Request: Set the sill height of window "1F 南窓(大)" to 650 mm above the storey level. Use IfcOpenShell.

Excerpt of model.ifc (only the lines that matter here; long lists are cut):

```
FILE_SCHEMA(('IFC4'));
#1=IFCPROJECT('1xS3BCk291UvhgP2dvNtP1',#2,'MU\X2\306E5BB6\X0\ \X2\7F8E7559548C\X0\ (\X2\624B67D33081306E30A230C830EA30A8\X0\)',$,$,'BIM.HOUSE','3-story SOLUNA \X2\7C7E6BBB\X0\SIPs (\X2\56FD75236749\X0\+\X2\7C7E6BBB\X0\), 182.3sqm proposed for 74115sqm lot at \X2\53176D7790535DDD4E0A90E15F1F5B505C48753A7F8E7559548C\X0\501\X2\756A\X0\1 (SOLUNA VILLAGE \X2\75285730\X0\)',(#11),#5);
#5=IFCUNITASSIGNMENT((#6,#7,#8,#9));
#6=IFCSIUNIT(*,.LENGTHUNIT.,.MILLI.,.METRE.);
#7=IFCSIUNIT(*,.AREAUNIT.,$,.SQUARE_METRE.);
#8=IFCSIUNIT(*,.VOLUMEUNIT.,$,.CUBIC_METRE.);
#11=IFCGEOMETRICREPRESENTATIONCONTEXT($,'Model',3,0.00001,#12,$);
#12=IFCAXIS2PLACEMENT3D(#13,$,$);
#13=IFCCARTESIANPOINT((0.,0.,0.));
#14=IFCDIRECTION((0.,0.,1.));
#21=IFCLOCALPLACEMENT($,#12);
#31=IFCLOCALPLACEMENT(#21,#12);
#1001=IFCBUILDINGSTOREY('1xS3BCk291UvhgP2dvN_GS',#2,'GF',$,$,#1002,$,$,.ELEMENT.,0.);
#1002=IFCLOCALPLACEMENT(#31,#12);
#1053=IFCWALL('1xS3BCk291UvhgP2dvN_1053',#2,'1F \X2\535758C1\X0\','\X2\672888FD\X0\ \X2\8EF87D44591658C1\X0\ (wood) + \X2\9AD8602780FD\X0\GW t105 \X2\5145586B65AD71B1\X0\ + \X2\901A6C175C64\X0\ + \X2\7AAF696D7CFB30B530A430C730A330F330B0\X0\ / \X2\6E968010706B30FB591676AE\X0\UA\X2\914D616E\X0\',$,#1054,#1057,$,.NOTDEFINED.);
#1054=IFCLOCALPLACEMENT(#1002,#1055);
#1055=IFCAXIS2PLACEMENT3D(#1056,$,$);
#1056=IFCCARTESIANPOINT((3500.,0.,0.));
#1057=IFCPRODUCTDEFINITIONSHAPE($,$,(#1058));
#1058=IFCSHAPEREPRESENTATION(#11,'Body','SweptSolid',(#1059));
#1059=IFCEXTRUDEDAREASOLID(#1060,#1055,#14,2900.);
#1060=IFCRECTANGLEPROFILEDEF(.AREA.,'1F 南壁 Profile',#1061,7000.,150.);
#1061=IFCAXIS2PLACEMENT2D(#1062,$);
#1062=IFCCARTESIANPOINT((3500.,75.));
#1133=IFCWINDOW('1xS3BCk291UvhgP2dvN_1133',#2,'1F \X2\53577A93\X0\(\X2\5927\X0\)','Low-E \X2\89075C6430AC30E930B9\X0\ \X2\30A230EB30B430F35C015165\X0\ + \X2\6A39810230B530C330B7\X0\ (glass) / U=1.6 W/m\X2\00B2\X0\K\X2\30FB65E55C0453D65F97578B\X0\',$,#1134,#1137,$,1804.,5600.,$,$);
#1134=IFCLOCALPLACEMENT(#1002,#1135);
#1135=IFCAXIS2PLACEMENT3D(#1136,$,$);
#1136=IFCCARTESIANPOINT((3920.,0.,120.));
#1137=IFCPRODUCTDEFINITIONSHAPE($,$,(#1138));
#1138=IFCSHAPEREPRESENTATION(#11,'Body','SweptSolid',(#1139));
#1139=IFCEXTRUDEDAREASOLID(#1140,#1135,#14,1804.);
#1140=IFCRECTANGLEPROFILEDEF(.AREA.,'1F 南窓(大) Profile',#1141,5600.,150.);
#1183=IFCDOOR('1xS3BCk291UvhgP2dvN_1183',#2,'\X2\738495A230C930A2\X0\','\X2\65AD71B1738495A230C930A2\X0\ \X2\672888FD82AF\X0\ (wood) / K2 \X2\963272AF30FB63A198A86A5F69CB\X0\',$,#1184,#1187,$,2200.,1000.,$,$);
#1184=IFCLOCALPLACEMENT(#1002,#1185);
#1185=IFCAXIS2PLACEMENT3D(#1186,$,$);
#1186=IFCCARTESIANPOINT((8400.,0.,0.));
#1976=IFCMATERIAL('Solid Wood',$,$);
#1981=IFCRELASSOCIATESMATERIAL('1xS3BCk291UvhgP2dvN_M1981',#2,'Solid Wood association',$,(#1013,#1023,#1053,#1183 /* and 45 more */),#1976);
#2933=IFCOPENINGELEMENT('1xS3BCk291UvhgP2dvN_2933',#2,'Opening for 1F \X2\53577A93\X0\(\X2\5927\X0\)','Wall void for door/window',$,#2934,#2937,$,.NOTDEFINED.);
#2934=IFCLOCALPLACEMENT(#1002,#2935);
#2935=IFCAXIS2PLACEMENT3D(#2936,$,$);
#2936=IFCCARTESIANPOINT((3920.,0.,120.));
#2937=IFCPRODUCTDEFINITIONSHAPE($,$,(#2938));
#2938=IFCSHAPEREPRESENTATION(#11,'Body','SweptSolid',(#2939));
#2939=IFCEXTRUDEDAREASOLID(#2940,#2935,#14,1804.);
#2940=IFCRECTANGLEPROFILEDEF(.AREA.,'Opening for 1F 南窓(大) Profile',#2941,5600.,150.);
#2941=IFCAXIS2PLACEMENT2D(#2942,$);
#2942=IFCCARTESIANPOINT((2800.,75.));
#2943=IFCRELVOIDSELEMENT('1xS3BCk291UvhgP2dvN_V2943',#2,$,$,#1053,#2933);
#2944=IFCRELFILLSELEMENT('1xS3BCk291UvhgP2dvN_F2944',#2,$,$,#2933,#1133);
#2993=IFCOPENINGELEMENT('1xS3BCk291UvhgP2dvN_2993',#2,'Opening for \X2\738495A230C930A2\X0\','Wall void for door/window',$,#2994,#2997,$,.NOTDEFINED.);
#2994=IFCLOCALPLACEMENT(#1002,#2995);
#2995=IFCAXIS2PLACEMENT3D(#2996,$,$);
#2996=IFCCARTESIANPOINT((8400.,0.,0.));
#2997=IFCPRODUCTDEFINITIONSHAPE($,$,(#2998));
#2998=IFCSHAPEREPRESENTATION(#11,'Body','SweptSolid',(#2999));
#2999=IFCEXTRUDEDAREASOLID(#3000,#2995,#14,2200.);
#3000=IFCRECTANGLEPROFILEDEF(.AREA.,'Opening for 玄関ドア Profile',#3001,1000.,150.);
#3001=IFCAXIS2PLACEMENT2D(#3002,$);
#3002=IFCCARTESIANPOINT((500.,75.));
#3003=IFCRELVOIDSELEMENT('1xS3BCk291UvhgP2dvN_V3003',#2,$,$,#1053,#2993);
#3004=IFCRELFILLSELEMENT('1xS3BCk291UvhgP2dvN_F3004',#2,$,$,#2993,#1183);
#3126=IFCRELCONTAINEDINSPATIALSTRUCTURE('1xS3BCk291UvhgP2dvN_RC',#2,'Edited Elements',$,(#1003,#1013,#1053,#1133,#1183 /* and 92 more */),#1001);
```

```python
import numpy as np
import ifcopenshell
import ifcopenshell.api.geometry
import ifcopenshell.geom
import ifcopenshell.util.element
import ifcopenshell.util.placement
import ifcopenshell.util.shape
import ifcopenshell.util.unit

model = ifcopenshell.open("model.ifc")
unit_scale = ifcopenshell.util.unit.calculate_unit_scale(model)

window = model.by_guid("1xS3BCk291UvhgP2dvN_1133")
opening = window.FillsVoids[0].RelatingOpeningElement
storey = ifcopenshell.util.element.get_container(window, ifc_class="IfcBuildingStorey")
level = ifcopenshell.util.placement.get_local_placement(storey.ObjectPlacement)[2, 3]

# The opening's origin need not be at the sill, so measure its lowest point.
shape = ifcopenshell.geom.create_shape(ifcopenshell.geom.settings(), opening)
bottom = ifcopenshell.util.shape.get_shape_bottom_elevation(shape, shape.geometry) / unit_scale
dz = level + 0.65 / unit_scale - bottom

shift = np.array([0.0, 0.0, dz])
# The window is not placed relative to its opening, so move both.
for product in (opening, window):
    matrix = ifcopenshell.util.placement.get_local_placement(product.ObjectPlacement)
    matrix[:3, 3] += shift
    ifcopenshell.api.geometry.edit_object_placement(model, product=product, matrix=matrix, is_si=False)

print(f"moved by {dz * unit_scale:+.3f} m")

model.write("model_edited.ifc")
```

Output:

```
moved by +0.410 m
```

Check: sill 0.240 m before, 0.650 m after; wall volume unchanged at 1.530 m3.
